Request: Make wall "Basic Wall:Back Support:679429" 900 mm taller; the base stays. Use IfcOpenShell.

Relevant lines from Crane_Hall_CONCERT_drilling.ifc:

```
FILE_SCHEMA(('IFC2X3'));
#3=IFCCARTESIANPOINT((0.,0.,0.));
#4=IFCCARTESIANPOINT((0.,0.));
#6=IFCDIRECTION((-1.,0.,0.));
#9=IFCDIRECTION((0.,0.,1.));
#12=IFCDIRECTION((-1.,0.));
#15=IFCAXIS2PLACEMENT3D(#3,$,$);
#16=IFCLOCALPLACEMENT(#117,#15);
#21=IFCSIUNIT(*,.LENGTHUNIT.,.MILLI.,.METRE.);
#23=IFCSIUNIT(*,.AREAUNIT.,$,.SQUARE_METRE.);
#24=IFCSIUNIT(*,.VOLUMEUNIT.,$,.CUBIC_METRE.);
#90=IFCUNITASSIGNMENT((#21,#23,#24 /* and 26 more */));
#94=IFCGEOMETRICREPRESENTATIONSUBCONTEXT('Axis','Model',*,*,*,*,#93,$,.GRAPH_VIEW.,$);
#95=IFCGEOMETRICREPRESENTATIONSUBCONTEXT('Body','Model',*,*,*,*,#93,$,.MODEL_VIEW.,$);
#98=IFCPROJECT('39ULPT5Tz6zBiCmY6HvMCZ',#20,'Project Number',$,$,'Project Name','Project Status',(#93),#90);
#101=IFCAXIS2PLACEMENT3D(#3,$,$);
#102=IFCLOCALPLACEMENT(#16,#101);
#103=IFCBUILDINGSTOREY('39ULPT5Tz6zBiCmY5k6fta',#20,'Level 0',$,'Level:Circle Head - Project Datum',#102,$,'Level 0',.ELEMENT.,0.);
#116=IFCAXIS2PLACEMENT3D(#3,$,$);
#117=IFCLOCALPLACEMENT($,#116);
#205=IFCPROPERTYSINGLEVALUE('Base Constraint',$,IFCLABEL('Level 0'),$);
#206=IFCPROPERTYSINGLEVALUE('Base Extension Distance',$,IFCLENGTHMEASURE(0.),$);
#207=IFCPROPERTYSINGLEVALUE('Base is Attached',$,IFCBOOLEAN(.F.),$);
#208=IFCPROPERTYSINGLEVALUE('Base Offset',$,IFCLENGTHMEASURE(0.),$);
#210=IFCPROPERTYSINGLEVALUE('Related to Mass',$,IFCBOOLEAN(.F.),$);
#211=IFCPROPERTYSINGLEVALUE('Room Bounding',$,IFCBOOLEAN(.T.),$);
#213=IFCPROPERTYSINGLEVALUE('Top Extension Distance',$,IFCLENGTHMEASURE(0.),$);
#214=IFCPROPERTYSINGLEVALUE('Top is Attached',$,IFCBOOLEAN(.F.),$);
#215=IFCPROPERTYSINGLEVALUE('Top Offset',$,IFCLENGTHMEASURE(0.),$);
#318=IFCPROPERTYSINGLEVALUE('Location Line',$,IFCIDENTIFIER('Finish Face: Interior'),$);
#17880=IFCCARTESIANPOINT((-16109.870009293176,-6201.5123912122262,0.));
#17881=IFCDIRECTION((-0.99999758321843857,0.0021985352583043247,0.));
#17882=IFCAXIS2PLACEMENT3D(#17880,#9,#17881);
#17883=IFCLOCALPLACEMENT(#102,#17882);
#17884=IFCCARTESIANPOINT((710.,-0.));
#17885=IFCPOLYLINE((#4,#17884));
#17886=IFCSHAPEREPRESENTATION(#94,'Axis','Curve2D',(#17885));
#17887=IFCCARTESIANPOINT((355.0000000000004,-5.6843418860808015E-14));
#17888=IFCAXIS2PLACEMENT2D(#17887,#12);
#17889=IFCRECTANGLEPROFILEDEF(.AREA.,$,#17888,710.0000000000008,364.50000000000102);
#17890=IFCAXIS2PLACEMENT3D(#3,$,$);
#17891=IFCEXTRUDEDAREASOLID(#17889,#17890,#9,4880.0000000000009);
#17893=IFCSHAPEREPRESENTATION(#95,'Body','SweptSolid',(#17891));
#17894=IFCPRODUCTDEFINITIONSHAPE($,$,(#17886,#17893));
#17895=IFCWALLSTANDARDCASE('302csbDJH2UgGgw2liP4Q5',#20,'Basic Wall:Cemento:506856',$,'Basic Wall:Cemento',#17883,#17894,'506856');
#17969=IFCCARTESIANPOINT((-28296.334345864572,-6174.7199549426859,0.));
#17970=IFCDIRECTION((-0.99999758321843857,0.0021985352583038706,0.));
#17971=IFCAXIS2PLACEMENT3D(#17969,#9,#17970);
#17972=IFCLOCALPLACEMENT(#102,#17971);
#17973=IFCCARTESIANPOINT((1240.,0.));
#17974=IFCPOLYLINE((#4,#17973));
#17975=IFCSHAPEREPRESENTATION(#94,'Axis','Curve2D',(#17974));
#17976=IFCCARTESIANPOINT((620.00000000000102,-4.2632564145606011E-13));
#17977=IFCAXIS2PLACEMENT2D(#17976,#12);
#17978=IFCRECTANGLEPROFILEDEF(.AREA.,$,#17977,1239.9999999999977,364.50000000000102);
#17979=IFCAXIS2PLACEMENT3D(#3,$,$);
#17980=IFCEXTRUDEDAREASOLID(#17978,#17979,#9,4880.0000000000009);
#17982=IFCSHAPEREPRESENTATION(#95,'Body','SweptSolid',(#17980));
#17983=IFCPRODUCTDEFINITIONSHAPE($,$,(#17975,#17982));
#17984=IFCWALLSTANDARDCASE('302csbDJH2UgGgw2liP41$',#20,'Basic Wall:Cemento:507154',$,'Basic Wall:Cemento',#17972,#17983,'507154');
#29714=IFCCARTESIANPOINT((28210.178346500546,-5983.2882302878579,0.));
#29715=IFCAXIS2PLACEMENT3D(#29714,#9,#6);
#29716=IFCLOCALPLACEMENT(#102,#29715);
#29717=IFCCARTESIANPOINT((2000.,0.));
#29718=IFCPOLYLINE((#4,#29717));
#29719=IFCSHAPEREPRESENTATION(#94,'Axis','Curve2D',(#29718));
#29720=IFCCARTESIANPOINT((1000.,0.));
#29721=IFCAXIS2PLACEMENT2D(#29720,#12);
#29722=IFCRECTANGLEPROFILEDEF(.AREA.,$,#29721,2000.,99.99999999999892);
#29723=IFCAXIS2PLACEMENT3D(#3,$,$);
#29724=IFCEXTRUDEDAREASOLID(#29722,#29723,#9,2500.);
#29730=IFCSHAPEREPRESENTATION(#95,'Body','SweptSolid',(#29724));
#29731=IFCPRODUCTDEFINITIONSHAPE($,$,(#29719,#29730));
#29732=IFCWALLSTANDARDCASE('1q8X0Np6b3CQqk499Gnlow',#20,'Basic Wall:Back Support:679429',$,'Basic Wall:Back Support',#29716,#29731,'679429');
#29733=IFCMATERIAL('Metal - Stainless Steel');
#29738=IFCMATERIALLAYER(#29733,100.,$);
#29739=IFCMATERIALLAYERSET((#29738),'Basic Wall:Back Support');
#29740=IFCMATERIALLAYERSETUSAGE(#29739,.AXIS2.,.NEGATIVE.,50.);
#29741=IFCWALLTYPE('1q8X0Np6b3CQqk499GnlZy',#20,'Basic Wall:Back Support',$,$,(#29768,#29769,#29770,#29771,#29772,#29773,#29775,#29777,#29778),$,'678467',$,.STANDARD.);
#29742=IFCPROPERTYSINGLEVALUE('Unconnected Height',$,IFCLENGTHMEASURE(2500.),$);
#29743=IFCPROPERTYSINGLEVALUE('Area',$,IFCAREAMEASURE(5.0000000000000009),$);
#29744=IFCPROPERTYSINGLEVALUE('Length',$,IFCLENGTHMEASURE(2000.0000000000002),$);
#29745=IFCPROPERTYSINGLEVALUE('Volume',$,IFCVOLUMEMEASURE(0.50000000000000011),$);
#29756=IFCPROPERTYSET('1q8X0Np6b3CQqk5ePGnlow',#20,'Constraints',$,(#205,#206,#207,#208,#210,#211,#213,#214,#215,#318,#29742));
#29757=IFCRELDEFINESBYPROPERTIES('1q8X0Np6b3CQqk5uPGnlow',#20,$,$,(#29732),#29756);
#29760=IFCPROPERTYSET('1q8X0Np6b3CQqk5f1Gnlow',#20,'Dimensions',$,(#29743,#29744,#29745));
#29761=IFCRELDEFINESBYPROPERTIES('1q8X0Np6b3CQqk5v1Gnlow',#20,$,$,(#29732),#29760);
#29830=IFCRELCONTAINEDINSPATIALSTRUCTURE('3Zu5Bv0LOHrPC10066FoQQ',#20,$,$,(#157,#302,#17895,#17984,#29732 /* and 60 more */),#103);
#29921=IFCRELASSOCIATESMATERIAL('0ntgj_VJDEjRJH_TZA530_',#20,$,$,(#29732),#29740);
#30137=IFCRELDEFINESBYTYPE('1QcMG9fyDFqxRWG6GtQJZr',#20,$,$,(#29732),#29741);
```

```python
import ifcopenshell
import ifcopenshell.api.pset
import ifcopenshell.geom
import ifcopenshell.util.element
import ifcopenshell.util.representation
import ifcopenshell.util.shape
import ifcopenshell.util.unit

model = ifcopenshell.open("Crane_Hall_CONCERT_drilling.ifc")
area_scale = ifcopenshell.util.unit.calculate_unit_scale(model, "AREAUNIT")
volume_scale = ifcopenshell.util.unit.calculate_unit_scale(model, "VOLUMEUNIT")
settings = ifcopenshell.geom.settings()


def volume(element):
    """Net volume in cubic metres, openings subtracted."""
    shape = ifcopenshell.geom.create_shape(settings, element)
    return ifcopenshell.util.shape.get_volume(shape.geometry)


wall = model.by_guid("1q8X0Np6b3CQqk499Gnlow")
before = volume(wall)

body = ifcopenshell.util.representation.get_representation(wall, "Model", "Body")
solid = body.Items[0]
old_height = solid.Depth
solid.Depth += 900.0
after = volume(wall)
thickness = 0.1  # wall thickness in metres

# Update the stored height, areas and volumes.
pset = model.by_id(ifcopenshell.util.element.get_pset(wall, "Constraints", should_inherit=False)["id"])
ifcopenshell.api.pset.edit_pset(model, pset=pset, properties={
    "Unconnected Height": model.create_entity("IfcLengthMeasure", solid.Depth),
})
pset = model.by_id(ifcopenshell.util.element.get_pset(wall, "Dimensions", should_inherit=False)["id"])
ifcopenshell.api.pset.edit_pset(model, pset=pset, properties={
    "Area": model.create_entity("IfcAreaMeasure", after / thickness / area_scale),
    "Volume": model.create_entity("IfcVolumeMeasure", after / volume_scale),
})

print(f"height {old_height:g} -> {solid.Depth:g}, volume {before:.3f} -> {after:.3f} m3")

model.write("Crane_Hall_CONCERT_drilling-out.ifc")
```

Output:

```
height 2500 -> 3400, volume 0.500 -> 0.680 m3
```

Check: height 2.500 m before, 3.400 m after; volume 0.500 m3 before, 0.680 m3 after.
